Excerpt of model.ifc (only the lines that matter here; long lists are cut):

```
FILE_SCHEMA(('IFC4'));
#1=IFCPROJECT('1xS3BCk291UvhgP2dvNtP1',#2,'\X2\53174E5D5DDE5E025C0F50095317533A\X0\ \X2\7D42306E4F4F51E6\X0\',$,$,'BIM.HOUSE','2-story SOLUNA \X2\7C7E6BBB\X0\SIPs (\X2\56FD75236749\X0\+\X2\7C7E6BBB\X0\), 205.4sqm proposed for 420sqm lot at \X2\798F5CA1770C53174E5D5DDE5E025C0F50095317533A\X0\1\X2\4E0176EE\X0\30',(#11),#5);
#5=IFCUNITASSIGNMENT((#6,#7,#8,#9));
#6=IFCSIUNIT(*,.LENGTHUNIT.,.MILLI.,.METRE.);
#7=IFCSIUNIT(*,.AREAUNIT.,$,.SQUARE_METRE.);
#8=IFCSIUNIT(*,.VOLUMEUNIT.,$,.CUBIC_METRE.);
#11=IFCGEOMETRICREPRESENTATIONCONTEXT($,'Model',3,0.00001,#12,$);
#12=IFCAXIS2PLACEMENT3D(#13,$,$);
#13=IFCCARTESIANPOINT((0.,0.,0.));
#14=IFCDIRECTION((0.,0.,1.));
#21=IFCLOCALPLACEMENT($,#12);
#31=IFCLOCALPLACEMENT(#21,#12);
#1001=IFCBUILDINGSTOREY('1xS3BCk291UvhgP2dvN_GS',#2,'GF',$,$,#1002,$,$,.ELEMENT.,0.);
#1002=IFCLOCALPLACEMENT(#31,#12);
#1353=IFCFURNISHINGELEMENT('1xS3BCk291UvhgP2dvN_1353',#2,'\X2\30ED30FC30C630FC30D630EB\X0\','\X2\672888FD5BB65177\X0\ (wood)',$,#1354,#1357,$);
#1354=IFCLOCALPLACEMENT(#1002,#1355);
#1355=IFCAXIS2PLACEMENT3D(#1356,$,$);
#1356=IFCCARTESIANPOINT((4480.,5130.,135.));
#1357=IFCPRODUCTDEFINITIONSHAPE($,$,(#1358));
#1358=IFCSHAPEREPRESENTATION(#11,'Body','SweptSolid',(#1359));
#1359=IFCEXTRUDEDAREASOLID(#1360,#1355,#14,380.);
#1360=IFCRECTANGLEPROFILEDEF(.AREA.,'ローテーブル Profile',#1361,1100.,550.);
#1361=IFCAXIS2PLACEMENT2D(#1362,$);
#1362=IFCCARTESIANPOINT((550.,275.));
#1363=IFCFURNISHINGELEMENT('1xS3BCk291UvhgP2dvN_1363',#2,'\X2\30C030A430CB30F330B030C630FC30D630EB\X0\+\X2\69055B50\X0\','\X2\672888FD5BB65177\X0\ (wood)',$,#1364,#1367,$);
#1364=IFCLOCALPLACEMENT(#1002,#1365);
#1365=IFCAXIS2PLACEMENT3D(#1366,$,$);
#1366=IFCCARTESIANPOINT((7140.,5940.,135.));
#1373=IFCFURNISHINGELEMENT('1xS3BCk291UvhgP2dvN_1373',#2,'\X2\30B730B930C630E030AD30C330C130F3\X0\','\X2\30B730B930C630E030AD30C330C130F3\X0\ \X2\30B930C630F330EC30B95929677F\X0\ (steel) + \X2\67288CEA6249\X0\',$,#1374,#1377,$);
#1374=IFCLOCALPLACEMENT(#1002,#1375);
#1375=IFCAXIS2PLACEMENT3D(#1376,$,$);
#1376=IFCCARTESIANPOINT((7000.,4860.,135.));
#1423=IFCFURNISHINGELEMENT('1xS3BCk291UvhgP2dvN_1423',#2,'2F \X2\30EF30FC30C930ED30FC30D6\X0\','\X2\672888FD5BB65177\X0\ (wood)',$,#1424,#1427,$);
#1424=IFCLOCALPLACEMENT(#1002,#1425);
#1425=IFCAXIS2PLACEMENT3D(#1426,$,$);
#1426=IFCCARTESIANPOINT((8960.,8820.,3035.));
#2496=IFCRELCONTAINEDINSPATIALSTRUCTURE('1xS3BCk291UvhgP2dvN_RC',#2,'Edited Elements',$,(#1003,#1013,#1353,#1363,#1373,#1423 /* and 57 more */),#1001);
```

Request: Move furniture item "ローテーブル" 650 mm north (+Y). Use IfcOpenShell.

```python
import ifcopenshell
import ifcopenshell.api.geometry
import ifcopenshell.util.placement
import ifcopenshell.util.unit

model = ifcopenshell.open("model.ifc")
unit_scale = ifcopenshell.util.unit.calculate_unit_scale(model)

item = model.by_guid("1xS3BCk291UvhgP2dvN_1353")
matrix = ifcopenshell.util.placement.get_local_placement(item.ObjectPlacement)
matrix[1, 3] += 0.65 / unit_scale
ifcopenshell.api.geometry.edit_object_placement(model, product=item, matrix=matrix, is_si=False)

print(ifcopenshell.util.placement.get_local_placement(item.ObjectPlacement).round(3) + 0.0)

model.write("model-out.ifc")
```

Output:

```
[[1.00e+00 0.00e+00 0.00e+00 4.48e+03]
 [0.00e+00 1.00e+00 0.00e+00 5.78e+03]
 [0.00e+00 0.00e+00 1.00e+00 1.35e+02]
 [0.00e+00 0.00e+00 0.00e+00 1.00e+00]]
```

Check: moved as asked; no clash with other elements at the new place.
